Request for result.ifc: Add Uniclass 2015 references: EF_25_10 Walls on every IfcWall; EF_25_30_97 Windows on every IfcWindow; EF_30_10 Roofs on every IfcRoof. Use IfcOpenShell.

First a look at what the model holds.

```python
import ifcopenshell

model = ifcopenshell.open("result.ifc")
print(model.schema)
print("classifications:", [c.Name for c in model.by_type("IfcClassification")])
for ifc_class in ("IfcDoor", "IfcRoof", "IfcStair", "IfcWall", "IfcWindow"):
    print(ifc_class, len(model.by_type(ifc_class)))
```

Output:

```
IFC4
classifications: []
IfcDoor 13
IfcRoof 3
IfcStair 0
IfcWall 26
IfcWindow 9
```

```python
import ifcopenshell
import ifcopenshell.api.classification

model = ifcopenshell.open("result.ifc")

system = ifcopenshell.api.classification.add_classification(model, classification="Uniclass 2015")

codes = {
    "IfcWall": ("EF_25_10", "Walls"),
    "IfcWindow": ("EF_25_30_97", "Windows"),
    "IfcRoof": ("EF_30_10", "Roofs"),
}
for ifc_class, (code, name) in codes.items():
    products = model.by_type(ifc_class)
    ifcopenshell.api.classification.add_reference(
        model, products=products, classification=system, identification=code, name=name
    )
    print(code, len(products))

model.write("result_updated.ifc")
```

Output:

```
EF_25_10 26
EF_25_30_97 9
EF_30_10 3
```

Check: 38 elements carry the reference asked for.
